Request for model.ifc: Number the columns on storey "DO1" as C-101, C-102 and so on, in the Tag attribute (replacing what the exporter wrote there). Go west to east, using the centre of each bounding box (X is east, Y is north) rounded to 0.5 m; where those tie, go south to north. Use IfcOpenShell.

First a look at what the model holds.

```python
import ifcopenshell
import ifcopenshell.util.element
import ifcopenshell.util.placement

model = ifcopenshell.open("model.ifc")
print(model.schema)
storey = next(s for s in model.by_type("IfcBuildingStorey") if s.Name == "DO1")
columns = [e for e in ifcopenshell.util.element.get_decomposition(storey) if e.is_a("IfcColumn")]
for e in sorted(columns, key=lambda e: e.id()):
    origin = ifcopenshell.util.placement.get_local_placement(e.ObjectPlacement)[:3, 3]
    print(e.id(), e.Tag, e.Name, origin.round(2) + 0.0, sep=" | ")
```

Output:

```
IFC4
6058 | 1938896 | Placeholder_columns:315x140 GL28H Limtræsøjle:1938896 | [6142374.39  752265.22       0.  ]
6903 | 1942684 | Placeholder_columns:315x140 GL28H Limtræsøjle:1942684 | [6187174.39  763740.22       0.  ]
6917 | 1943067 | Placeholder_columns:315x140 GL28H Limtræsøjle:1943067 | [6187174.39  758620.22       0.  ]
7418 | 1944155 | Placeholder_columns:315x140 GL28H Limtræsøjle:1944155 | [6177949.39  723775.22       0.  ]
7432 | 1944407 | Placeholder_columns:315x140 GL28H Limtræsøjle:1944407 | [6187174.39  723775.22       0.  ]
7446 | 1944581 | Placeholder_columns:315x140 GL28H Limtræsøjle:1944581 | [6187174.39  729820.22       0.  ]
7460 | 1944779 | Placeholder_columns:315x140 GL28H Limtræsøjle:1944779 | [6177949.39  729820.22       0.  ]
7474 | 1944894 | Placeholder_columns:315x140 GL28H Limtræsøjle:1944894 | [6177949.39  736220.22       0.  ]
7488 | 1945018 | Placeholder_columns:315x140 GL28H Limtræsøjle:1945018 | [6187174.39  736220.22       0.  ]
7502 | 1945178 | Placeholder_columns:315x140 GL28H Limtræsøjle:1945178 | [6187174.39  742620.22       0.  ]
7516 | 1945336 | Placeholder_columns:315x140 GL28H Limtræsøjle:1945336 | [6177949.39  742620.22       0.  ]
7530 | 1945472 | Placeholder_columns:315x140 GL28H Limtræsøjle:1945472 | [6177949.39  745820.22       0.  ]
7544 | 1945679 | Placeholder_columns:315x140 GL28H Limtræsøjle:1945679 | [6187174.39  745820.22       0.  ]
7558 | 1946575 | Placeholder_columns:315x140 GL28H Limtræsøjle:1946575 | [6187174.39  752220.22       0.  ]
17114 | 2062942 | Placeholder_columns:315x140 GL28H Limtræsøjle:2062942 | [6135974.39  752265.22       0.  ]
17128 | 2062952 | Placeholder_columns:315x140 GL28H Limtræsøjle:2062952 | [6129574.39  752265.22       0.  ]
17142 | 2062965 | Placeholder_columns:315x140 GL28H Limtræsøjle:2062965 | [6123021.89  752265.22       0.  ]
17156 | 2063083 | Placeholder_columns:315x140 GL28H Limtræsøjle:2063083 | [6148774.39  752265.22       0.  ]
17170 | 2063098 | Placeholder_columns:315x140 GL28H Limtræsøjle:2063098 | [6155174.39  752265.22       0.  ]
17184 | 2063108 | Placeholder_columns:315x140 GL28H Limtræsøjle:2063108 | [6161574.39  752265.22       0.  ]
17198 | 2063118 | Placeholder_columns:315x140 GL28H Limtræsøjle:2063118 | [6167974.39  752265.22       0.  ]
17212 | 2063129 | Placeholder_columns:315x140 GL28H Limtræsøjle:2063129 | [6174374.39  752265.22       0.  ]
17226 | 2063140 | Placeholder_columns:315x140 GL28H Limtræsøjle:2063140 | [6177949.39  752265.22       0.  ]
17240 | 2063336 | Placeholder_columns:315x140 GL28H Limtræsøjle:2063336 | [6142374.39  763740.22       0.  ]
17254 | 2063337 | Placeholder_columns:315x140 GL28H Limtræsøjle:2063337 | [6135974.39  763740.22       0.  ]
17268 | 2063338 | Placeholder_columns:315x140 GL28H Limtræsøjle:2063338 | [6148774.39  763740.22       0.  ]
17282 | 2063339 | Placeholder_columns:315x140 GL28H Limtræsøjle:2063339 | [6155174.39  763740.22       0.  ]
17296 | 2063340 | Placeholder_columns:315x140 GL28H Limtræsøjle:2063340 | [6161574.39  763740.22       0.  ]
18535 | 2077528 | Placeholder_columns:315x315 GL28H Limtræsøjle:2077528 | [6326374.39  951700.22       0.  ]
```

```python
import ifcopenshell
import ifcopenshell.geom
import ifcopenshell.util.element
import ifcopenshell.util.shape

model = ifcopenshell.open("model.ifc")
settings = ifcopenshell.geom.settings()
settings.set("use-world-coords", True)


def centre(element):
    shape = ifcopenshell.geom.create_shape(settings, element)
    return ifcopenshell.util.shape.get_bbox_centroid(shape.geometry)


storey = next(s for s in model.by_type("IfcBuildingStorey") if s.Name == "DO1")
columns = [e for e in ifcopenshell.util.element.get_decomposition(storey) if e.is_a("IfcColumn")]

# Insertion points can sit at a corner or the storey origin, so sort by the geometry (in metres).
centres = {e: centre(e) for e in columns}
columns.sort(key=lambda e: (round(centres[e][0] / 0.5), centres[e][1]))

for i, e in enumerate(columns, start=1):
    number = f"C-1{i:02d}"
    e.Tag = number
    print(e.id(), number)

model.write("model_updated.ifc")
```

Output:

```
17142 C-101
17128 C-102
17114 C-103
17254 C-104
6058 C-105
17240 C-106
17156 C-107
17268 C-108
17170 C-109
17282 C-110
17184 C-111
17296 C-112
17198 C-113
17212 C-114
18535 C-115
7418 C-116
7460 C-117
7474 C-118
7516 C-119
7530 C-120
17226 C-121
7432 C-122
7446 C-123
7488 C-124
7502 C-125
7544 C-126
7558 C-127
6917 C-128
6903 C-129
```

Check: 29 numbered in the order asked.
